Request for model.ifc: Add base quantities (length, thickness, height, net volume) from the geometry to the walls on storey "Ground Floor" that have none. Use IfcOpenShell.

First a look at what the model holds.

```python
import ifcopenshell
import ifcopenshell.util.element
import ifcopenshell.util.unit

model = ifcopenshell.open("model.ifc")
print(model.schema)
for unit_type in ("LENGTHUNIT", "AREAUNIT", "VOLUMEUNIT"):
    print(unit_type, ifcopenshell.util.unit.calculate_unit_scale(model, unit_type))
storey = next(s for s in model.by_type("IfcBuildingStorey") if s.Name == "Ground Floor")
walls = [e for e in ifcopenshell.util.element.get_decomposition(storey) if e.is_a("IfcWall")]
for e in sorted(walls, key=lambda e: e.id()):
    print(e.id(), e.is_a(), e.Name, list(ifcopenshell.util.element.get_psets(e, qtos_only=True)), sep=" | ")
```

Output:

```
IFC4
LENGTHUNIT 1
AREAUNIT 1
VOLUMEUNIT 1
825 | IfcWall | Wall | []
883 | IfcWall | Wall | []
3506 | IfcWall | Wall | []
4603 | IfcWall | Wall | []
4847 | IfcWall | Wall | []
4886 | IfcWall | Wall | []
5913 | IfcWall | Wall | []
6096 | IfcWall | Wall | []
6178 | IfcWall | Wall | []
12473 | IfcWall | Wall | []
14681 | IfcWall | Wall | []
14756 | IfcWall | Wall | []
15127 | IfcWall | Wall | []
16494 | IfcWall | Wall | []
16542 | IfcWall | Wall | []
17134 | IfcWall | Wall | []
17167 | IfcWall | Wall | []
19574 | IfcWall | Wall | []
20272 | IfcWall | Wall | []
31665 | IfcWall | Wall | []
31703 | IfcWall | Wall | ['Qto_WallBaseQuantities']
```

```python
import ifcopenshell
import ifcopenshell.api.pset
import ifcopenshell.geom
import ifcopenshell.util.element
import ifcopenshell.util.shape
import ifcopenshell.util.unit

model = ifcopenshell.open("model.ifc")
unit_scale = ifcopenshell.util.unit.calculate_unit_scale(model)
volume_scale = ifcopenshell.util.unit.calculate_unit_scale(model, "VOLUMEUNIT")
settings = ifcopenshell.geom.settings()

storey = next(s for s in model.by_type("IfcBuildingStorey") if s.Name == "Ground Floor")
walls = [e for e in ifcopenshell.util.element.get_decomposition(storey) if e.is_a("IfcWall")]

for e in sorted(walls, key=lambda e: e.id()):
    if ifcopenshell.util.element.get_psets(e, qtos_only=True, should_inherit=False):
        continue
    # Geometry comes back in metres, in the element's own axes.
    shape = ifcopenshell.geom.create_shape(settings, e)
    values = {
        "Length": ifcopenshell.util.shape.get_x(shape.geometry) / unit_scale,
        "Width": ifcopenshell.util.shape.get_y(shape.geometry) / unit_scale,
        "Height": ifcopenshell.util.shape.get_z(shape.geometry) / unit_scale,
        "NetVolume": ifcopenshell.util.shape.get_volume(shape.geometry) / volume_scale,
    }
    qto = ifcopenshell.api.pset.add_qto(model, product=e, name="Qto_WallBaseQuantities")
    ifcopenshell.api.pset.edit_qto(model, qto=qto, properties=values)
    print(e.id(), {k: round(v, 3) for k, v in values.items()})

model.write("model-out.ifc")
```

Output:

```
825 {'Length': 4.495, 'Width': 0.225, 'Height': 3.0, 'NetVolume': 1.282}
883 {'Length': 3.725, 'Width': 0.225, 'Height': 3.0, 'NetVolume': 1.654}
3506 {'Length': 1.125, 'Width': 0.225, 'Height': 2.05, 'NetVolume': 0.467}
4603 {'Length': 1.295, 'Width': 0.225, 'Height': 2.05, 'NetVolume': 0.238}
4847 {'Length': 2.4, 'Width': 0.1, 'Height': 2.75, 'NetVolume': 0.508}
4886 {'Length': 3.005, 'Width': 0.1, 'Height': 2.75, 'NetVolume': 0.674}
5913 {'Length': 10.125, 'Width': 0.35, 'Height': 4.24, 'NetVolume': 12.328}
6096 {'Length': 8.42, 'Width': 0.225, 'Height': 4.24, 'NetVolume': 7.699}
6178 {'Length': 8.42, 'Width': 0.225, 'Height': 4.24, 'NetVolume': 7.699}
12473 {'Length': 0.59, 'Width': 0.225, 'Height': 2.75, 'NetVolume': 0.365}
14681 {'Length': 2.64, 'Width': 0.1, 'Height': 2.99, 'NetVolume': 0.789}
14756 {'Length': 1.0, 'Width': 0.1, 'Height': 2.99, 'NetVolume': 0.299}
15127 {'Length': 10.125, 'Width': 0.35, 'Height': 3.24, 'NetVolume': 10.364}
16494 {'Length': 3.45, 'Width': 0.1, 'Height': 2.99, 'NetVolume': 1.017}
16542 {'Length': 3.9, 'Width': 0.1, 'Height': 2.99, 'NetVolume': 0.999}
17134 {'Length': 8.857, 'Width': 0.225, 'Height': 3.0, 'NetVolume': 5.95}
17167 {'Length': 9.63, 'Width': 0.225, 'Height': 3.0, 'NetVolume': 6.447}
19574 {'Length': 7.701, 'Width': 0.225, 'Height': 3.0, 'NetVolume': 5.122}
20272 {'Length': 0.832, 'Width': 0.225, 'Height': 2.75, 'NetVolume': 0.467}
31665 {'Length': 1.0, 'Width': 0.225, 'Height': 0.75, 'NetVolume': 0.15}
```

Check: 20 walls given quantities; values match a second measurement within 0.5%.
